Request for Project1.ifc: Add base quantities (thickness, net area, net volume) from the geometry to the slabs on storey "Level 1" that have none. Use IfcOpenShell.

First a look at what the model holds.

```python
import ifcopenshell
import ifcopenshell.util.element
import ifcopenshell.util.unit

model = ifcopenshell.open("Project1.ifc")
print(model.schema)
for unit_type in ("LENGTHUNIT", "AREAUNIT", "VOLUMEUNIT"):
    print(unit_type, ifcopenshell.util.unit.calculate_unit_scale(model, unit_type))
storey = next(s for s in model.by_type("IfcBuildingStorey") if s.Name == "Level 1")
slabs = [e for e in ifcopenshell.util.element.get_decomposition(storey) if e.is_a("IfcSlab")]
for e in sorted(slabs, key=lambda e: e.id()):
    print(e.id(), e.is_a(), e.Name, list(ifcopenshell.util.element.get_psets(e, qtos_only=True)), sep=" | ")
```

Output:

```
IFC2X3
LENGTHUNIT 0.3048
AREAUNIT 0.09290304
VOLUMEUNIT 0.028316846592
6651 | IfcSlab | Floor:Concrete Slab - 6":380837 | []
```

```python
import ifcopenshell
import ifcopenshell.api.pset
import ifcopenshell.geom
import ifcopenshell.util.element
import ifcopenshell.util.shape
import ifcopenshell.util.unit

model = ifcopenshell.open("Project1.ifc")
unit_scale = ifcopenshell.util.unit.calculate_unit_scale(model)
area_scale = ifcopenshell.util.unit.calculate_unit_scale(model, "AREAUNIT")
volume_scale = ifcopenshell.util.unit.calculate_unit_scale(model, "VOLUMEUNIT")
settings = ifcopenshell.geom.settings()

storey = next(s for s in model.by_type("IfcBuildingStorey") if s.Name == "Level 1")
slabs = [e for e in ifcopenshell.util.element.get_decomposition(storey) if e.is_a("IfcSlab")]

for e in sorted(slabs, key=lambda e: e.id()):
    if ifcopenshell.util.element.get_psets(e, qtos_only=True, should_inherit=False):
        continue
    # Geometry comes back in metres, in the element's own axes.
    shape = ifcopenshell.geom.create_shape(settings, e)
    values = {
        "Width": ifcopenshell.util.shape.get_z(shape.geometry) / unit_scale,
        "NetArea": ifcopenshell.util.shape.get_footprint_area(shape.geometry) / area_scale,
        "NetVolume": ifcopenshell.util.shape.get_volume(shape.geometry) / volume_scale,
    }
    qto = ifcopenshell.api.pset.add_qto(model, product=e, name="BaseQuantities")
    ifcopenshell.api.pset.edit_qto(model, qto=qto, properties=values)
    print(e.id(), {k: round(v, 3) for k, v in values.items()})

model.write("Project1_v2.ifc")
```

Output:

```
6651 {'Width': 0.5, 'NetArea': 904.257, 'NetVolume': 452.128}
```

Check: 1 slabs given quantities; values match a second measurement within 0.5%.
